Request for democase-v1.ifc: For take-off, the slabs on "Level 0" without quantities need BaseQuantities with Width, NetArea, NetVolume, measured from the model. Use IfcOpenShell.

First a look at what the model holds.

```python
import ifcopenshell
import ifcopenshell.util.element
import ifcopenshell.util.unit

model = ifcopenshell.open("democase-v1.ifc")
print(model.schema)
for unit_type in ("LENGTHUNIT", "AREAUNIT", "VOLUMEUNIT"):
    print(unit_type, ifcopenshell.util.unit.calculate_unit_scale(model, unit_type))
storey = next(s for s in model.by_type("IfcBuildingStorey") if s.Name == "Level 0")
slabs = [e for e in ifcopenshell.util.element.get_decomposition(storey) if e.is_a("IfcSlab")]
for e in sorted(slabs, key=lambda e: e.id()):
    print(e.id(), e.is_a(), e.Name, list(ifcopenshell.util.element.get_psets(e, qtos_only=True)), sep=" | ")
```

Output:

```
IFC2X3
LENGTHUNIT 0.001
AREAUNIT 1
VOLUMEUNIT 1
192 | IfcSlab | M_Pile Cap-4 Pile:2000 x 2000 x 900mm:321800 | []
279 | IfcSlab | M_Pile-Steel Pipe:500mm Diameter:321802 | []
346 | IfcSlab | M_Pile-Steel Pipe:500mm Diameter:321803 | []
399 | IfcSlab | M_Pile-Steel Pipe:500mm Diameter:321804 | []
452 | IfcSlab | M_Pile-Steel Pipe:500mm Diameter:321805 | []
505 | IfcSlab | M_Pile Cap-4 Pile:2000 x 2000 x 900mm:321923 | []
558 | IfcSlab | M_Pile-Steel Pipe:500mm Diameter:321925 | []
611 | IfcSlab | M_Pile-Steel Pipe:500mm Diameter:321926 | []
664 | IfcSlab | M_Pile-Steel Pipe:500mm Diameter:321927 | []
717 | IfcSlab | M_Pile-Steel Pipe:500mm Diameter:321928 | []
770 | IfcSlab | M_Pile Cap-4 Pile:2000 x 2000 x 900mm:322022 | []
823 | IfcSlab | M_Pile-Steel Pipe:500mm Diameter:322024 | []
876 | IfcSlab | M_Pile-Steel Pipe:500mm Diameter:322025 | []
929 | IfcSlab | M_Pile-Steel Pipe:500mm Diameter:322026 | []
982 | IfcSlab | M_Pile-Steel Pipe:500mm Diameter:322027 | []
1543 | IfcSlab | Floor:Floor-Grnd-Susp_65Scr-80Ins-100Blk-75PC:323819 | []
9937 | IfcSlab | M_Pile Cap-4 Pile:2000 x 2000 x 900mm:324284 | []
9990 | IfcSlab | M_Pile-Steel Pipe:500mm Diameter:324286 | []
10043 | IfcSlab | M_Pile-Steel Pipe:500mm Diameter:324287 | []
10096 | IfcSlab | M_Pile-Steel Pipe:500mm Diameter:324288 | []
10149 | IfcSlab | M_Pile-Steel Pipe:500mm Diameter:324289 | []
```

```python
import ifcopenshell
import ifcopenshell.api.pset
import ifcopenshell.geom
import ifcopenshell.util.element
import ifcopenshell.util.shape
import ifcopenshell.util.unit

model = ifcopenshell.open("democase-v1.ifc")
unit_scale = ifcopenshell.util.unit.calculate_unit_scale(model)
area_scale = ifcopenshell.util.unit.calculate_unit_scale(model, "AREAUNIT")
volume_scale = ifcopenshell.util.unit.calculate_unit_scale(model, "VOLUMEUNIT")
settings = ifcopenshell.geom.settings()

storey = next(s for s in model.by_type("IfcBuildingStorey") if s.Name == "Level 0")
slabs = [e for e in ifcopenshell.util.element.get_decomposition(storey) if e.is_a("IfcSlab")]

for e in sorted(slabs, key=lambda e: e.id()):
    if ifcopenshell.util.element.get_psets(e, qtos_only=True, should_inherit=False):
        continue
    # Geometry comes back in metres, in the element's own axes.
    shape = ifcopenshell.geom.create_shape(settings, e)
    values = {
        "Width": ifcopenshell.util.shape.get_z(shape.geometry) / unit_scale,
        "NetArea": ifcopenshell.util.shape.get_footprint_area(shape.geometry) / area_scale,
        "NetVolume": ifcopenshell.util.shape.get_volume(shape.geometry) / volume_scale,
    }
    qto = ifcopenshell.api.pset.add_qto(model, product=e, name="BaseQuantities")
    ifcopenshell.api.pset.edit_qto(model, qto=qto, properties=values)
    print(e.id(), {k: round(v, 3) for k, v in values.items()})

model.write("democase-v1_rev.ifc")
```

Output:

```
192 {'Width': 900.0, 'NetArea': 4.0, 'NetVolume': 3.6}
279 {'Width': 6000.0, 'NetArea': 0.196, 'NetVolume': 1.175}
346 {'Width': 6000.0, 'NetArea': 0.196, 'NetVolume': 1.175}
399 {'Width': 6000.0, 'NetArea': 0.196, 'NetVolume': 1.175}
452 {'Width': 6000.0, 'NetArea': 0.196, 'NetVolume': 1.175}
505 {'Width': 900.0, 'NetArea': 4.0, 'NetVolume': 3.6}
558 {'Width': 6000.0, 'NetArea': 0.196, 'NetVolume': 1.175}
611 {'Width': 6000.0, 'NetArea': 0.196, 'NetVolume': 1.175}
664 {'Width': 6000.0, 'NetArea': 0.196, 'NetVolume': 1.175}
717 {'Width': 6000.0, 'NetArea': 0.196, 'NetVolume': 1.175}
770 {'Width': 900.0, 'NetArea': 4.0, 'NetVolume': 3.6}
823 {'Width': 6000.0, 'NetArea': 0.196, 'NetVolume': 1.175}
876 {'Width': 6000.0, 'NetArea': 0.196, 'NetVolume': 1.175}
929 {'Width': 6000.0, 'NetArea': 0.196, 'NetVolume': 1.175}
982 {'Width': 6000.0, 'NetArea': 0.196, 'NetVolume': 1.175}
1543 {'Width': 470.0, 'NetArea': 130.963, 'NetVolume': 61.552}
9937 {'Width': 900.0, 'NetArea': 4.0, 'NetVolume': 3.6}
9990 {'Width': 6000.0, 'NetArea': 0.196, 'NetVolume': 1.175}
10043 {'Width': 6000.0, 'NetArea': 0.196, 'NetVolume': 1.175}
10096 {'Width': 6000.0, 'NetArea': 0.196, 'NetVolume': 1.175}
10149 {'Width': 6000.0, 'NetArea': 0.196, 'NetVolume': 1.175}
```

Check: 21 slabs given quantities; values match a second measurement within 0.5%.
